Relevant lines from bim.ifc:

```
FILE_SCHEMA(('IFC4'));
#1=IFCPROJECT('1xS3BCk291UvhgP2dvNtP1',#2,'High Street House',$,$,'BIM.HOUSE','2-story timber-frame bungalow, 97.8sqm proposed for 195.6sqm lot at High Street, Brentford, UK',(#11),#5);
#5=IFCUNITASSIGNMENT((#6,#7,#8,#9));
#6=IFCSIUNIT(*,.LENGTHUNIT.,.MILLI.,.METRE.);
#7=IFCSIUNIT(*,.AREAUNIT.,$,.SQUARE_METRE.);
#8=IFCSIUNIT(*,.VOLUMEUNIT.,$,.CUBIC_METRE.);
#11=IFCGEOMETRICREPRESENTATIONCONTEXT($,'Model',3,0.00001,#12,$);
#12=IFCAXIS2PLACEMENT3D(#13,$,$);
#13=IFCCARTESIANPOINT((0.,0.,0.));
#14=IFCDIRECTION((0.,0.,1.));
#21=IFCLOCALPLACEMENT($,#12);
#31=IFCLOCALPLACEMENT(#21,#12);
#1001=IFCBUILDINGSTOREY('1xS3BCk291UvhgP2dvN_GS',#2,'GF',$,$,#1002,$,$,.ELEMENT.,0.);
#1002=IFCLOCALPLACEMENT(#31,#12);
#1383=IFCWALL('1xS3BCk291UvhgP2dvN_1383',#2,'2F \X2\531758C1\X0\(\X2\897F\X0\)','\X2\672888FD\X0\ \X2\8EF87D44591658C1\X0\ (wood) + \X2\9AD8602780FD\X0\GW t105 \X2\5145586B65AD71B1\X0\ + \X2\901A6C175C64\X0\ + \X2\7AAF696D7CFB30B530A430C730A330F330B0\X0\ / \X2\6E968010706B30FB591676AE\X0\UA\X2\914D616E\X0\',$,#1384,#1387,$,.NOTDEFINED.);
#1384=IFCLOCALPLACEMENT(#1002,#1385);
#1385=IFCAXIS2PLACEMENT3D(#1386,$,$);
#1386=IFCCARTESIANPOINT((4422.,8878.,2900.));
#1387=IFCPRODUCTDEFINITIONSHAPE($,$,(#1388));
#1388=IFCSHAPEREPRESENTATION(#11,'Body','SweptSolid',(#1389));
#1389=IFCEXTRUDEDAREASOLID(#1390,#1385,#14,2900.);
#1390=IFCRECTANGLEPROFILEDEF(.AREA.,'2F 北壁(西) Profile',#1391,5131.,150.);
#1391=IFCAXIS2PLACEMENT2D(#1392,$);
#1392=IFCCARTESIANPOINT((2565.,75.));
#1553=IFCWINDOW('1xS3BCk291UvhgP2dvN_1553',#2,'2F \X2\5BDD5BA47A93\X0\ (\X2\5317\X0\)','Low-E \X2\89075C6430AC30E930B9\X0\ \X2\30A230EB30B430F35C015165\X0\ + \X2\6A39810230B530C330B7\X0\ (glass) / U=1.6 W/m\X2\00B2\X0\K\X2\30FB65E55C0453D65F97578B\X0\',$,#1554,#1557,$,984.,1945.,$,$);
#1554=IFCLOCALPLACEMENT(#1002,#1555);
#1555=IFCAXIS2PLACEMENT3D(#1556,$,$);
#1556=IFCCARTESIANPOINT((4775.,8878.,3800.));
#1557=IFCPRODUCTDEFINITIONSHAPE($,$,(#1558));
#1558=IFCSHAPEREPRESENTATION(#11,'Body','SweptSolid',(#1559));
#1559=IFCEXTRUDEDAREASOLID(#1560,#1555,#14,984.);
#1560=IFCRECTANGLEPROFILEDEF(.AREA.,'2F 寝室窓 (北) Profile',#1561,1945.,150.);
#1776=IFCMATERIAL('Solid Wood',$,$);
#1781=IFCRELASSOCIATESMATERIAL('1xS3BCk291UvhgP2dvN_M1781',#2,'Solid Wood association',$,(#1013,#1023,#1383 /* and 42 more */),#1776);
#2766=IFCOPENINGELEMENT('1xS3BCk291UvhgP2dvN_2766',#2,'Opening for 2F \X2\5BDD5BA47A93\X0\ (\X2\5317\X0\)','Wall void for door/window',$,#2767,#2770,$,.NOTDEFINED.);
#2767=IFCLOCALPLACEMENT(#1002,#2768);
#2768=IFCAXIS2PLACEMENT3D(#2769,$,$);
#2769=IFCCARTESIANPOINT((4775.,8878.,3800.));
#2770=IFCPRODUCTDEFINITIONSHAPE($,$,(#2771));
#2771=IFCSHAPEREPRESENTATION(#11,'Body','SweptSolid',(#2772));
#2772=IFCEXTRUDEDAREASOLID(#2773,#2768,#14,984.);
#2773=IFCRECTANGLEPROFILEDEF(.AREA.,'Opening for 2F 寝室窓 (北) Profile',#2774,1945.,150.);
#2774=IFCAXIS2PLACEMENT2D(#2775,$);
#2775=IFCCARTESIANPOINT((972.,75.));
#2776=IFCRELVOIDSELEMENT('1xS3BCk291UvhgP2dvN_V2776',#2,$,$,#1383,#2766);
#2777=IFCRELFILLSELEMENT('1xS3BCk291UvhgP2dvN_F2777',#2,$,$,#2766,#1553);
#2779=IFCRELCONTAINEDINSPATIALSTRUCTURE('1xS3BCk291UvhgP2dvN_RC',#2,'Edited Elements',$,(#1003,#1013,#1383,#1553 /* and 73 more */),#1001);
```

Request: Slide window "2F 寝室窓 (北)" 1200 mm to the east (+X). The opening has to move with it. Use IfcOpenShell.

```python
import ifcopenshell
import ifcopenshell.api.geometry
import ifcopenshell.util.placement
import ifcopenshell.util.unit

model = ifcopenshell.open("bim.ifc")
unit_scale = ifcopenshell.util.unit.calculate_unit_scale(model)

window = model.by_id(1553)
opening = window.FillsVoids[0].RelatingOpeningElement
wall = opening.VoidsElements[0].RelatingBuildingElement

wall_matrix = ifcopenshell.util.placement.get_local_placement(wall.ObjectPlacement)
shift = wall_matrix[:3, 0] * 1.2 / unit_scale
before = ifcopenshell.util.placement.get_local_placement(window.ObjectPlacement)[:3, 3].copy()

# The window is not placed relative to its opening, so move both.
for product in (opening, window):
    matrix = ifcopenshell.util.placement.get_local_placement(product.ObjectPlacement)
    matrix[:3, 3] += shift
    ifcopenshell.api.geometry.edit_object_placement(model, product=product, matrix=matrix, is_si=False)

after = ifcopenshell.util.placement.get_local_placement(window.ObjectPlacement)[:3, 3]
print("window moved by", (after - before).round(3) + 0.0)

model.write("bim-out.ifc")
```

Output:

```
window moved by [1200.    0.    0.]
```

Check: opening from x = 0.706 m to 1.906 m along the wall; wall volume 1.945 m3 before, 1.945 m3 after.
